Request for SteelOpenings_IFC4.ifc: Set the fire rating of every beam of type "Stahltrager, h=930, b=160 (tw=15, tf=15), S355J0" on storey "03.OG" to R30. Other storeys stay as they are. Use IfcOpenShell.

First a look at what the model holds.

```python
import ifcopenshell
import ifcopenshell.util.element

model = ifcopenshell.open("SteelOpenings_IFC4.ifc")
print(model.schema)
storey = next(s for s in model.by_type("IfcBuildingStorey") if s.Name == "03.OG")
beams = [e for e in ifcopenshell.util.element.get_decomposition(storey) if e.is_a("IfcBeam")]
seen = {}
for e in beams:
    element_type = ifcopenshell.util.element.get_type(e)
    key = (element_type.Name if element_type != e and element_type else None, ifcopenshell.util.element.get_pset(e, "Pset_BeamCommon", "FireRating"))
    seen[key] = seen.get(key, 0) + 1
for (name, value), count in sorted(seen.items(), key=str):
    print(count, "x", name, "|", value)
```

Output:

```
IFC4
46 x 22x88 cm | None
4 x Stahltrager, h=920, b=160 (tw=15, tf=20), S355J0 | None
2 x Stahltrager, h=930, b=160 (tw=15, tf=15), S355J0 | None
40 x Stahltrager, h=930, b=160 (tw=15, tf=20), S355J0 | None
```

```python
import ifcopenshell
import ifcopenshell.api.pset
import ifcopenshell.util.element

model = ifcopenshell.open("SteelOpenings_IFC4.ifc")

storey = next(s for s in model.by_type("IfcBuildingStorey") if s.Name == "03.OG")
beams = [e for e in ifcopenshell.util.element.get_decomposition(storey) if e.is_a("IfcBeam")]

count = 0
for e in beams:
    element_type = ifcopenshell.util.element.get_type(e)
    if element_type in (None, e) or element_type.Name != "Stahltrager, h=930, b=160 (tw=15, tf=15), S355J0":
        continue
    # add_pset returns the element's existing set when there is one.
    pset = ifcopenshell.api.pset.add_pset(model, product=e, name="Pset_BeamCommon")
    ifcopenshell.api.pset.edit_pset(model, pset=pset, properties={"FireRating": "R30"})
    count += 1

print(count, "beams updated")

model.write("SteelOpenings_IFC4_rev.ifc")
```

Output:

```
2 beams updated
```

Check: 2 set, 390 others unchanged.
